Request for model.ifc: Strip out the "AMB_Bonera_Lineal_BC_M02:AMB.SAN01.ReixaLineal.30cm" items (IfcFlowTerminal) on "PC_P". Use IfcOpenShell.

First a look at what the model holds.

```python
import ifcopenshell
import ifcopenshell.util.element

model = ifcopenshell.open("model.ifc")
print(model.schema)
storey = next(s for s in model.by_type("IfcBuildingStorey") if s.Name == "PC_P")
terminals = [e for e in ifcopenshell.util.element.get_decomposition(storey) if e.is_a("IfcFlowTerminal")]
seen = {}
for e in terminals:
    element_type = ifcopenshell.util.element.get_type(e)
    name = element_type.Name if element_type not in (None, e) else None
    seen[name] = seen.get(name, 0) + 1
for name, count in sorted(seen.items(), key=str):
    print(count, "x", name)
```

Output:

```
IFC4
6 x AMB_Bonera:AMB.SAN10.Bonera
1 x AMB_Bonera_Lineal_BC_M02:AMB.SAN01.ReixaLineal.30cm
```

```python
import ifcopenshell
import ifcopenshell.api.root
import ifcopenshell.util.element

model = ifcopenshell.open("model.ifc")

storey = next(s for s in model.by_type("IfcBuildingStorey") if s.Name == "PC_P")
terminals = [e for e in ifcopenshell.util.element.get_decomposition(storey) if e.is_a("IfcFlowTerminal")]
targets = [e for e in terminals if (t := ifcopenshell.util.element.get_type(e)) not in (None, e) and t.Name == "AMB_Bonera_Lineal_BC_M02:AMB.SAN01.ReixaLineal.30cm"]

for e in targets:
    ifcopenshell.api.root.remove_product(model, product=e)
print(len(targets), "removed")

model.write("model_v2.ifc")
```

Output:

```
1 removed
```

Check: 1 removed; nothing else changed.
